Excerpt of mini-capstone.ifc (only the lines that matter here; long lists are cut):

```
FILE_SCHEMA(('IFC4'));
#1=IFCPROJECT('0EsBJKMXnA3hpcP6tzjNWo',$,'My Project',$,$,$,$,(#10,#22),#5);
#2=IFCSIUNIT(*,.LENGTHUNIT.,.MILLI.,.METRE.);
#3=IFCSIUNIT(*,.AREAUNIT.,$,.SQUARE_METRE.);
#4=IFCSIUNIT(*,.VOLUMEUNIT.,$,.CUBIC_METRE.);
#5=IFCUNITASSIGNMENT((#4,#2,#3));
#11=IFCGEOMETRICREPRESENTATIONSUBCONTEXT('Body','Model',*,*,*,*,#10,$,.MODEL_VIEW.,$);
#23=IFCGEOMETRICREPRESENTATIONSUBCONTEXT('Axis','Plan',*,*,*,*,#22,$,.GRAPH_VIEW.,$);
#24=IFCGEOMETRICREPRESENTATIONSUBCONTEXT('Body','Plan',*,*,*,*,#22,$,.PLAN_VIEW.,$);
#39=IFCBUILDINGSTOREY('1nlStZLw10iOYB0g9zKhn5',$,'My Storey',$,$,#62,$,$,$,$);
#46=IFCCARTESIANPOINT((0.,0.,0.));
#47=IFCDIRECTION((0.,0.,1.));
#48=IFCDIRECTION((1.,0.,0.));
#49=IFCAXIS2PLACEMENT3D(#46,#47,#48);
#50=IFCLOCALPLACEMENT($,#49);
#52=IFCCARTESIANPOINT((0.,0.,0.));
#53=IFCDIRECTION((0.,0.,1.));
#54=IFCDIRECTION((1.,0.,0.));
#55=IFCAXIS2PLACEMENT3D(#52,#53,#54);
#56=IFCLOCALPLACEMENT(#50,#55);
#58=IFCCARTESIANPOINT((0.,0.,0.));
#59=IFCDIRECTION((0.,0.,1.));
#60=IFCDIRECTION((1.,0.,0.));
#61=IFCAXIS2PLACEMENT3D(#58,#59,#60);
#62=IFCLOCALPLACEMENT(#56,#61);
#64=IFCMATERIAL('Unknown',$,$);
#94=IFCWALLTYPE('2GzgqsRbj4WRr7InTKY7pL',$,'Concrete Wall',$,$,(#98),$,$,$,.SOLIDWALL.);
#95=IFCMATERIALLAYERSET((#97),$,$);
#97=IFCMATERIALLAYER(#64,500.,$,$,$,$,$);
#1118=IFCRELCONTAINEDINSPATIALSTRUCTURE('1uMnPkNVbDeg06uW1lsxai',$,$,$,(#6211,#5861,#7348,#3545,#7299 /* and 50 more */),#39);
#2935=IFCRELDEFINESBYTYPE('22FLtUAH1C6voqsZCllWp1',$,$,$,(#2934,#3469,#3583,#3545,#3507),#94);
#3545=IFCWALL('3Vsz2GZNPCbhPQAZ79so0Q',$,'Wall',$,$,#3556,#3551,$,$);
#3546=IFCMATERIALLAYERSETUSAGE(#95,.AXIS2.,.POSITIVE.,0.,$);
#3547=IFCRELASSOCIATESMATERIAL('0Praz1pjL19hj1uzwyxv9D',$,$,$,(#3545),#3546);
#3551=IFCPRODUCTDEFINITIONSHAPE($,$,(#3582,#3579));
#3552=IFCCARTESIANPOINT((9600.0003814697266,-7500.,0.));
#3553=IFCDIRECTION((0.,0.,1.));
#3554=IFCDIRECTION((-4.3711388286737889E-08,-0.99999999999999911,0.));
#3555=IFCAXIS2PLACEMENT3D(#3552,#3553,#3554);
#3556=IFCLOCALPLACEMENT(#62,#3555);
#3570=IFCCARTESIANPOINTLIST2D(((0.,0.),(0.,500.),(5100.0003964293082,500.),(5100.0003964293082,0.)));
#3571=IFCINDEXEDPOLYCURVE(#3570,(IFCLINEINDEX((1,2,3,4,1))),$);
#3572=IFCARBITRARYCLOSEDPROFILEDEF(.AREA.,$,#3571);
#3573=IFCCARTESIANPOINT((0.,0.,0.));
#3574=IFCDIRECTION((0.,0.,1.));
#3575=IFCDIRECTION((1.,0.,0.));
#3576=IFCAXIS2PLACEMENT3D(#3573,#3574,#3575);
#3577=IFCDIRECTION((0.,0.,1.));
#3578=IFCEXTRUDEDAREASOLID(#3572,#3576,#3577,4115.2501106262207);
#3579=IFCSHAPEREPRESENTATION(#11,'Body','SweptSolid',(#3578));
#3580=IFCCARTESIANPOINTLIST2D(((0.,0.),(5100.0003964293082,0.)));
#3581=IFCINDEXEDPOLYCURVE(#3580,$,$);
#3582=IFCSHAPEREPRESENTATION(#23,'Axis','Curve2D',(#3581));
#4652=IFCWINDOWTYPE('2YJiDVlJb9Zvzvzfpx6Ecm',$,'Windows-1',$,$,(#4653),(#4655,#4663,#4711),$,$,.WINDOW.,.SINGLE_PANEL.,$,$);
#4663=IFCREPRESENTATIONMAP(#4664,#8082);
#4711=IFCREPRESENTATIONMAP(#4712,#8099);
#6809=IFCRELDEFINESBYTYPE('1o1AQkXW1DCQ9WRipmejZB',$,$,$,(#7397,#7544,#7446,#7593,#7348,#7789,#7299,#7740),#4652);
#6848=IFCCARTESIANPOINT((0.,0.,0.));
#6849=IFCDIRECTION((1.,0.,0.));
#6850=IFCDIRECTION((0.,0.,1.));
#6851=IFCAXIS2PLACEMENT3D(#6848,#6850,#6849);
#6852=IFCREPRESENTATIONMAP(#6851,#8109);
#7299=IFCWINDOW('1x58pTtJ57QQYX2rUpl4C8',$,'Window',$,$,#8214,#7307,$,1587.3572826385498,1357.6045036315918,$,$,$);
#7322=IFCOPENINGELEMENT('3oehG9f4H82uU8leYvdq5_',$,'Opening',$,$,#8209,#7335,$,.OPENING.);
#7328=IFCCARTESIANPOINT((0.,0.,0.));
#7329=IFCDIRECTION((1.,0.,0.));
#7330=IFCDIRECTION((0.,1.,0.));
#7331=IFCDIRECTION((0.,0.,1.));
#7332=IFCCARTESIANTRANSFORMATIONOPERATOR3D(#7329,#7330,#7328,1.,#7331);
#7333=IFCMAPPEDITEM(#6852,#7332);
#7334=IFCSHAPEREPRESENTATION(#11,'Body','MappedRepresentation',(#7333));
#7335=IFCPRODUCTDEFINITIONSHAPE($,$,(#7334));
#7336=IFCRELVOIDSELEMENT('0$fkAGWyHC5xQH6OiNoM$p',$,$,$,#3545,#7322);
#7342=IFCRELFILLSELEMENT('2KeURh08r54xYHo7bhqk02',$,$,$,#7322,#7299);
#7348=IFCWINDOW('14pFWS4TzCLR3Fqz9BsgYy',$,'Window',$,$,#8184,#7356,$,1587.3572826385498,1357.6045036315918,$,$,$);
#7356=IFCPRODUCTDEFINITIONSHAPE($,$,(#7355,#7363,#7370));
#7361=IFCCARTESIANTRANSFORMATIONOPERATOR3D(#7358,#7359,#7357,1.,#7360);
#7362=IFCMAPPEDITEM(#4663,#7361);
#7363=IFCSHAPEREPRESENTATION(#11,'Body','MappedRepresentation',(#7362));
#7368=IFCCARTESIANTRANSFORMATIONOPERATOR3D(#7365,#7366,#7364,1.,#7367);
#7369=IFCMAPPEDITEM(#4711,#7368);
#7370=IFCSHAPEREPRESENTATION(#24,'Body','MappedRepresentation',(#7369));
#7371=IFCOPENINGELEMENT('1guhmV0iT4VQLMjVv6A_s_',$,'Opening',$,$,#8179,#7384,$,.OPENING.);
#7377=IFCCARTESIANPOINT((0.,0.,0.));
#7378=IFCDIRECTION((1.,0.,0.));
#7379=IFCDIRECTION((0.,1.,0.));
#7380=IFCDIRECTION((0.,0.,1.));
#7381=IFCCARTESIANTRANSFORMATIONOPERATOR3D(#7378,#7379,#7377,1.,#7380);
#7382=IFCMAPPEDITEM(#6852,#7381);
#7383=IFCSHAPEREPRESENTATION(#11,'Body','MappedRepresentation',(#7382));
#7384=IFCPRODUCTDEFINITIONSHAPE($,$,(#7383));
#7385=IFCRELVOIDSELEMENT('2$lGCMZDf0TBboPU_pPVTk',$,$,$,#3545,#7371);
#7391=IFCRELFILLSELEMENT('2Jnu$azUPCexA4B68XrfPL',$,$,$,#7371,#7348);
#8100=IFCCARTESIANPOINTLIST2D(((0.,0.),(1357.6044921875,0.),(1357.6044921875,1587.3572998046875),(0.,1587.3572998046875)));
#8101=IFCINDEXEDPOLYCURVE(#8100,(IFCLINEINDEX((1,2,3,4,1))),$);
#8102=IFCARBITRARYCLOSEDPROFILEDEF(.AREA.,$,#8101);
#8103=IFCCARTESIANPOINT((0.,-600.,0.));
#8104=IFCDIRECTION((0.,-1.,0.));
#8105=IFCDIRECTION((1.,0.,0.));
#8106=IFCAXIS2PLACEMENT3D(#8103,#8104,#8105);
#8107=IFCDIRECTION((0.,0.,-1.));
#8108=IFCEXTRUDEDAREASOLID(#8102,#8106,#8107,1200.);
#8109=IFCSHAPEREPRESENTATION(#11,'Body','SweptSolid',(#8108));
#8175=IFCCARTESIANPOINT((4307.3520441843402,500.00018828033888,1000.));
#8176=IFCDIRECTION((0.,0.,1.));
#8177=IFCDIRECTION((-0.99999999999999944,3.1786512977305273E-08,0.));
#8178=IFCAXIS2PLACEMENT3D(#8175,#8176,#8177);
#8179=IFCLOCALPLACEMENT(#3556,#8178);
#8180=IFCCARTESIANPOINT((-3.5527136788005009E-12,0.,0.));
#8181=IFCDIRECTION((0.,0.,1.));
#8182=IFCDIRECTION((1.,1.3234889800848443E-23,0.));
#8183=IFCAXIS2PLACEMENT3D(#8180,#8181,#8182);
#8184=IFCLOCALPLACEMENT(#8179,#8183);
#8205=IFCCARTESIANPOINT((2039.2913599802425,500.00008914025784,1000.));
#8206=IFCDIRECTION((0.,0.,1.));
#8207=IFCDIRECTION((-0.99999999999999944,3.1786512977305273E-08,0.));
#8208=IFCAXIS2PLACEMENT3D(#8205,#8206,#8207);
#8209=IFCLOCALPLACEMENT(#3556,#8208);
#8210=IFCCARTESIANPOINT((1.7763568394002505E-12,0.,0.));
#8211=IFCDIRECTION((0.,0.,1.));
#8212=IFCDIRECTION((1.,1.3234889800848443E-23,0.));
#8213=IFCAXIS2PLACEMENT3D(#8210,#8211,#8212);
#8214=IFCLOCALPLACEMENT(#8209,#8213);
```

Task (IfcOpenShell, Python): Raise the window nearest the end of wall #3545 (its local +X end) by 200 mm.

```python
import numpy as np
import ifcopenshell
import ifcopenshell.api.geometry
import ifcopenshell.util.placement
import ifcopenshell.util.unit

model = ifcopenshell.open("mini-capstone.ifc")
unit_scale = ifcopenshell.util.unit.calculate_unit_scale(model)

window = model.by_guid("14pFWS4TzCLR3Fqz9BsgYy")
opening = window.FillsVoids[0].RelatingOpeningElement
dz = 0.2 / unit_scale

shift = np.array([0.0, 0.0, dz])
# The window is placed relative to its opening, so it follows when the opening moves.
matrix = ifcopenshell.util.placement.get_local_placement(opening.ObjectPlacement)
matrix[:3, 3] += shift
ifcopenshell.api.geometry.edit_object_placement(
    model, product=opening, matrix=matrix, is_si=False, should_transform_children=True
)

print(f"moved by {dz * unit_scale:+.3f} m")

model.write("mini-capstone_edited.ifc")
```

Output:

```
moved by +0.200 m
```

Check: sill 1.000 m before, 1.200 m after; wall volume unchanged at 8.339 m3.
